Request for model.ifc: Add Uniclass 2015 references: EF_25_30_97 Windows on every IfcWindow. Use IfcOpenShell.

First a look at what the model holds.

```python
import ifcopenshell

model = ifcopenshell.open("model.ifc")
print(model.schema)
print("classifications:", [c.Name for c in model.by_type("IfcClassification")])
for ifc_class in ("IfcDoor", "IfcRoof", "IfcStair", "IfcWall", "IfcWindow"):
    print(ifc_class, len(model.by_type(ifc_class)))
```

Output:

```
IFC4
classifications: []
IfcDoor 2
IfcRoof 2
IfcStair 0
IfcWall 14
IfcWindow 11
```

```python
import ifcopenshell
import ifcopenshell.api.classification

model = ifcopenshell.open("model.ifc")

system = ifcopenshell.api.classification.add_classification(model, classification="Uniclass 2015")

codes = {
    "IfcWindow": ("EF_25_30_97", "Windows"),
}
for ifc_class, (code, name) in codes.items():
    products = model.by_type(ifc_class)
    ifcopenshell.api.classification.add_reference(
        model, products=products, classification=system, identification=code, name=name
    )
    print(code, len(products))

model.write("model_rev.ifc")
```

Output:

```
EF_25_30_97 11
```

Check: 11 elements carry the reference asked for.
